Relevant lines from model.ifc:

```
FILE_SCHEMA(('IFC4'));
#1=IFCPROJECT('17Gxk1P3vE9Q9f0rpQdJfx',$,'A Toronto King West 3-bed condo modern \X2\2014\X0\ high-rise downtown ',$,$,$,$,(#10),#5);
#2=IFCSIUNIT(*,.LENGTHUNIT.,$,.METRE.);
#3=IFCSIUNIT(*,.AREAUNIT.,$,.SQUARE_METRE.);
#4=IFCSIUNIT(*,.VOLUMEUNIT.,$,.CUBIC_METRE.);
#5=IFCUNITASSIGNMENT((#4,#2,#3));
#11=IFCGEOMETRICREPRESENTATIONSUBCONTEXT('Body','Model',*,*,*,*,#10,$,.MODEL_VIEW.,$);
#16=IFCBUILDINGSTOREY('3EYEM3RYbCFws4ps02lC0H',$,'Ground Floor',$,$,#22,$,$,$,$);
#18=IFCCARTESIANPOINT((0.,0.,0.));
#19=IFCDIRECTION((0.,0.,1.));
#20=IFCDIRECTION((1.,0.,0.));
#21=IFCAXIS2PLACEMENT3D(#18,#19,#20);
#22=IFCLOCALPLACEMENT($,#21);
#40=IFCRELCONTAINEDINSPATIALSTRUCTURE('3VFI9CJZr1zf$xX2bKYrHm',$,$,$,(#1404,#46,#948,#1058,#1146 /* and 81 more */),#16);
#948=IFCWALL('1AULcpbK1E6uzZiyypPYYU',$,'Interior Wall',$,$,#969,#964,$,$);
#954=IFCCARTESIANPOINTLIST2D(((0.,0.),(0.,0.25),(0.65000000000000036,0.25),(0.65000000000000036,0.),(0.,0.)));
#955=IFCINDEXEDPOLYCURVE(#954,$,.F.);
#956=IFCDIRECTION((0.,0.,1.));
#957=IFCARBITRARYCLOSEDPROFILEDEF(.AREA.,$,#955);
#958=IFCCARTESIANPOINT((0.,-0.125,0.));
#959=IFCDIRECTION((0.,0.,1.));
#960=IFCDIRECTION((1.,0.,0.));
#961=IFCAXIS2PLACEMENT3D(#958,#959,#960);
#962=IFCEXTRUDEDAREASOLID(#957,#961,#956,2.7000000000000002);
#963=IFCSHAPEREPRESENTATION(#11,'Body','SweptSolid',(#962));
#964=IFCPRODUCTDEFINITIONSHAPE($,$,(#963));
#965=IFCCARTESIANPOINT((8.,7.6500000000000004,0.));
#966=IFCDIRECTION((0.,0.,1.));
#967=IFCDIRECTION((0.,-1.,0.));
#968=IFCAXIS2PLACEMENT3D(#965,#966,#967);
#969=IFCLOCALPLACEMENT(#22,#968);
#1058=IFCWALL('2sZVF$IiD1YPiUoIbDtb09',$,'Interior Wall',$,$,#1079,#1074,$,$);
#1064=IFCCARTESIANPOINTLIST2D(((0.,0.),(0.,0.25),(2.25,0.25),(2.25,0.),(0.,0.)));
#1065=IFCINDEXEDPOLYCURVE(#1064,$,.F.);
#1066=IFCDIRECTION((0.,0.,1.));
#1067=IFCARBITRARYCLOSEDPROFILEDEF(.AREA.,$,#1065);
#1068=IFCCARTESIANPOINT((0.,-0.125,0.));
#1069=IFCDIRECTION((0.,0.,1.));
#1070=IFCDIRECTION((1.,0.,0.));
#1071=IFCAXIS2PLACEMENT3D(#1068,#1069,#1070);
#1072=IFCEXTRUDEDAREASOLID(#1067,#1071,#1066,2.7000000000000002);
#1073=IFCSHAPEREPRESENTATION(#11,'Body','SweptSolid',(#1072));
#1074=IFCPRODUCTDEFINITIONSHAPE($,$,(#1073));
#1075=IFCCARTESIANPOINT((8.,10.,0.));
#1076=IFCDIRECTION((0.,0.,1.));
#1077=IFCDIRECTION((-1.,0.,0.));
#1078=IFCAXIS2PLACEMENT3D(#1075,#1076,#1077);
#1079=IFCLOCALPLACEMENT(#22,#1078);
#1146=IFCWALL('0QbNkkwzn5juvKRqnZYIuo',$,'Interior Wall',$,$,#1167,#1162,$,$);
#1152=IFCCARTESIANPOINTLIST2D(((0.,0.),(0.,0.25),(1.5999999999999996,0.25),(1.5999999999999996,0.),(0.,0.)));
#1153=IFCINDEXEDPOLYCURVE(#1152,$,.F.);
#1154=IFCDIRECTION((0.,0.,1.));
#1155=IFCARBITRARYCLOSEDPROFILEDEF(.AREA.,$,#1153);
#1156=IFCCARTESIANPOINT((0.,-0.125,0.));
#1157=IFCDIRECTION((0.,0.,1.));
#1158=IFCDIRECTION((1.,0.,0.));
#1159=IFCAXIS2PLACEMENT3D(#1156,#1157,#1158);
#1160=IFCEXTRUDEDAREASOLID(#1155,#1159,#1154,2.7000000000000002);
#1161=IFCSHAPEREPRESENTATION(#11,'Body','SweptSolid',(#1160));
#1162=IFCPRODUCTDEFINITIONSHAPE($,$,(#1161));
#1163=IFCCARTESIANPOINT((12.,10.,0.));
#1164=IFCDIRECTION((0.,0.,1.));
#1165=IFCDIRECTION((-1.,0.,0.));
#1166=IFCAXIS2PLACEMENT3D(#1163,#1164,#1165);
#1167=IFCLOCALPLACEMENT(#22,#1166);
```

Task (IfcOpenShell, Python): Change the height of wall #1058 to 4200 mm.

```python
import ifcopenshell
import ifcopenshell.geom
import ifcopenshell.util.representation
import ifcopenshell.util.shape

model = ifcopenshell.open("model.ifc")
settings = ifcopenshell.geom.settings()


def volume(element):
    """Net volume in cubic metres, openings subtracted."""
    shape = ifcopenshell.geom.create_shape(settings, element)
    return ifcopenshell.util.shape.get_volume(shape.geometry)


wall = model.by_guid("2sZVF$IiD1YPiUoIbDtb09")
before = volume(wall)

body = ifcopenshell.util.representation.get_representation(wall, "Model", "Body")
solid = body.Items[0]
old_height = solid.Depth
solid.Depth = 4.2
after = volume(wall)

print(f"height {old_height:g} -> {solid.Depth:g}, volume {before:.3f} -> {after:.3f} m3")

model.write("model-out.ifc")
```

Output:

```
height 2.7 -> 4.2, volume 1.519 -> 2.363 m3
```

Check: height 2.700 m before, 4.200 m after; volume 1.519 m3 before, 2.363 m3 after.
